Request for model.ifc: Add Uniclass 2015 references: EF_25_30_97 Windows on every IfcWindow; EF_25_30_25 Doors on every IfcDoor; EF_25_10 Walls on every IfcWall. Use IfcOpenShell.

First a look at what the model holds.

```python
import ifcopenshell

model = ifcopenshell.open("model.ifc")
print(model.schema)
print("classifications:", [c.Name for c in model.by_type("IfcClassification")])
for ifc_class in ("IfcDoor", "IfcRoof", "IfcStair", "IfcWall", "IfcWindow"):
    print(ifc_class, len(model.by_type(ifc_class)))
```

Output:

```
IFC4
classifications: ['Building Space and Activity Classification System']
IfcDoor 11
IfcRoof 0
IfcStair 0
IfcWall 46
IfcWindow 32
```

```python
import ifcopenshell
import ifcopenshell.api.classification

model = ifcopenshell.open("model.ifc")

system = ifcopenshell.api.classification.add_classification(model, classification="Uniclass 2015")

codes = {
    "IfcWindow": ("EF_25_30_97", "Windows"),
    "IfcDoor": ("EF_25_30_25", "Doors"),
    "IfcWall": ("EF_25_10", "Walls"),
}
for ifc_class, (code, name) in codes.items():
    products = model.by_type(ifc_class)
    ifcopenshell.api.classification.add_reference(
        model, products=products, classification=system, identification=code, name=name
    )
    print(code, len(products))

model.write("model_edited.ifc")
```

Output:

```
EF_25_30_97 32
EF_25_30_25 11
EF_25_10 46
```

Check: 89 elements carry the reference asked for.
